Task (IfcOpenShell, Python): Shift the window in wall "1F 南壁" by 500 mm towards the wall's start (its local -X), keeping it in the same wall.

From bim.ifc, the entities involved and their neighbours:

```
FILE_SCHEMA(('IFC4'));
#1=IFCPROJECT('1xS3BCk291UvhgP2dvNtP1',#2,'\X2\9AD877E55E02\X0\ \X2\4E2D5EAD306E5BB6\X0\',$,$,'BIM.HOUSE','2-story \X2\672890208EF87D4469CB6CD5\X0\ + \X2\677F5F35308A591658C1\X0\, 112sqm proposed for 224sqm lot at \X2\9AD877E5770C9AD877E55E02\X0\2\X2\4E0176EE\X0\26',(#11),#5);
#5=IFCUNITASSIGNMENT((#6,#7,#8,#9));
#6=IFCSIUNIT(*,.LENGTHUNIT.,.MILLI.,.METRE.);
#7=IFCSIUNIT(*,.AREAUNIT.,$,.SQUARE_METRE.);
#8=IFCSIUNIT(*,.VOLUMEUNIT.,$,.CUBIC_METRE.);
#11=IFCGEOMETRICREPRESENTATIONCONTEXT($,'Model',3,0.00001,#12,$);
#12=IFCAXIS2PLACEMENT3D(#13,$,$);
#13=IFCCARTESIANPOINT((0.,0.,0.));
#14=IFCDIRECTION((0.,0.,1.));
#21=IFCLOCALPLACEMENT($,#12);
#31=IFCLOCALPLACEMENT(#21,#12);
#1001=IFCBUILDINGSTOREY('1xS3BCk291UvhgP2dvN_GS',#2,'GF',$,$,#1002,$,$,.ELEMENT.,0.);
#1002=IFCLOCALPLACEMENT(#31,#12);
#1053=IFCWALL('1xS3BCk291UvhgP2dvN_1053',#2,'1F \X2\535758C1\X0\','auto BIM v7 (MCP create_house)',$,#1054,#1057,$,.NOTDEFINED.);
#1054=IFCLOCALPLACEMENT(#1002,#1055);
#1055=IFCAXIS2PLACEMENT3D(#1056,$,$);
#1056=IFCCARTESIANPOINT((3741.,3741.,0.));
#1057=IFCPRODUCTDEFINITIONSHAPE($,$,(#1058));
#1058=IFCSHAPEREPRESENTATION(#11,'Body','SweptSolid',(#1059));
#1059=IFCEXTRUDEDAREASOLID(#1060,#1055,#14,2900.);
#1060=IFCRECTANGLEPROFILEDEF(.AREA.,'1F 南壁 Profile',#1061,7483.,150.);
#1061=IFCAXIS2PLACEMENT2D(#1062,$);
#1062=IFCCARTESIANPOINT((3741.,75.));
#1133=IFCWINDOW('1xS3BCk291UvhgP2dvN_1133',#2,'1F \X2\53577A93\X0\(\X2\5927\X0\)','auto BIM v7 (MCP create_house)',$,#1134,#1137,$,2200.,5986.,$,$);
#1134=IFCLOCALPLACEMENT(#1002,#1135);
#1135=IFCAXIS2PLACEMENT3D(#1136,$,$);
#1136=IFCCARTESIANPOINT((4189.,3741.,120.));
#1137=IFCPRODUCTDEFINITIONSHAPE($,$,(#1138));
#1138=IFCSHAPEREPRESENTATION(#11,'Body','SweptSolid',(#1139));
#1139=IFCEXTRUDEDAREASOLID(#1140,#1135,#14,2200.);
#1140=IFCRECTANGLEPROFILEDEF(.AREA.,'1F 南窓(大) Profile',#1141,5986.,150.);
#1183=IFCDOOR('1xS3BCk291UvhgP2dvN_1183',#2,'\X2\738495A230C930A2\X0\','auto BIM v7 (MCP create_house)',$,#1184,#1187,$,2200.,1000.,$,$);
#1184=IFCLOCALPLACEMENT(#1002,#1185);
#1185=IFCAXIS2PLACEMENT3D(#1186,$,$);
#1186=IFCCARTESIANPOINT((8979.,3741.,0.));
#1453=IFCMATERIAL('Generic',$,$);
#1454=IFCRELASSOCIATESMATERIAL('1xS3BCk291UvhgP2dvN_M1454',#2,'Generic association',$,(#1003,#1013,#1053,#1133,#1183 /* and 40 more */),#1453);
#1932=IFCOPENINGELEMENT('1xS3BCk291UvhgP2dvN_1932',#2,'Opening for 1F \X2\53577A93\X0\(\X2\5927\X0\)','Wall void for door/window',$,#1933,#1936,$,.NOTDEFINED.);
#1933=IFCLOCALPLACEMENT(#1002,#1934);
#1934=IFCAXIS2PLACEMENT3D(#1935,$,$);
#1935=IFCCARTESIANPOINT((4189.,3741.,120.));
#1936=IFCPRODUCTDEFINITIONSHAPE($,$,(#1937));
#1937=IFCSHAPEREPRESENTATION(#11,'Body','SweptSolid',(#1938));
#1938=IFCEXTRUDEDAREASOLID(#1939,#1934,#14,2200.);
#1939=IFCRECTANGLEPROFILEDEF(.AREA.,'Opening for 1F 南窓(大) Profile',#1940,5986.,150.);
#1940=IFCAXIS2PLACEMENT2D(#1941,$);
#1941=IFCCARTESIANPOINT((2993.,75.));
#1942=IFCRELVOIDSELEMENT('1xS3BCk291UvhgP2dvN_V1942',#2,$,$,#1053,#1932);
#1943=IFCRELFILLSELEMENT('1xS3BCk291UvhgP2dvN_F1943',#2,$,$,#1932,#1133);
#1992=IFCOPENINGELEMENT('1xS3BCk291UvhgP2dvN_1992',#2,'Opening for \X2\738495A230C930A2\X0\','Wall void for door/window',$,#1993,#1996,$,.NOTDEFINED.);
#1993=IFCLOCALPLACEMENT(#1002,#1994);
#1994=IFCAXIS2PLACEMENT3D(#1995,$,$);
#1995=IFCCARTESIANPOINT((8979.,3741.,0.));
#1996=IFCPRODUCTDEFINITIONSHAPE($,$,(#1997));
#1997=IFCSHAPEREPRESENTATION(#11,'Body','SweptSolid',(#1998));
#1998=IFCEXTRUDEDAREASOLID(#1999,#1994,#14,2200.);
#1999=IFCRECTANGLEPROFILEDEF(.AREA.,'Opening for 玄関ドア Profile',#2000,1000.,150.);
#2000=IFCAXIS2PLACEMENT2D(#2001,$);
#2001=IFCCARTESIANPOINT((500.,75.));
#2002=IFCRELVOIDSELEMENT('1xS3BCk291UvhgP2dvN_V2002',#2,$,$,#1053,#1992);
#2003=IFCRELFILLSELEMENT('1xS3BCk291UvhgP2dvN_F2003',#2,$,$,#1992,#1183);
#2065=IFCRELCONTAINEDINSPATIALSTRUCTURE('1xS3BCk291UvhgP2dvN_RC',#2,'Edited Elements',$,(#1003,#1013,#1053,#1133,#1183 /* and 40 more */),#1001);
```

```python
import ifcopenshell
import ifcopenshell.api.geometry
import ifcopenshell.util.placement

model = ifcopenshell.open("bim.ifc")

window = model.by_id(1133)
opening = window.FillsVoids[0].RelatingOpeningElement
wall = opening.VoidsElements[0].RelatingBuildingElement

wall_matrix = ifcopenshell.util.placement.get_local_placement(wall.ObjectPlacement)
shift = wall_matrix[:3, 0] * -500.0
before = ifcopenshell.util.placement.get_local_placement(window.ObjectPlacement)[:3, 3].copy()

# The window is not placed relative to its opening, so move both.
for product in (opening, window):
    matrix = ifcopenshell.util.placement.get_local_placement(product.ObjectPlacement)
    matrix[:3, 3] += shift
    ifcopenshell.api.geometry.edit_object_placement(model, product=product, matrix=matrix, is_si=False)

after = ifcopenshell.util.placement.get_local_placement(window.ObjectPlacement)[:3, 3]
print("window moved by", (after - before).round(3) + 0.0)

model.write("bim_edited.ifc")
```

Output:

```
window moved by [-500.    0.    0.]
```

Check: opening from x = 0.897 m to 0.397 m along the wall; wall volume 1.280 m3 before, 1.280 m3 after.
